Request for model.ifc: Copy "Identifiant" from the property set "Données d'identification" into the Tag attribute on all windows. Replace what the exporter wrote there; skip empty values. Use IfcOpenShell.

First a look at what the model holds.

```python
import ifcopenshell
import ifcopenshell.util.element

model = ifcopenshell.open("model.ifc")
print(model.schema)
windows = model.by_type("IfcWindow")
print(len(windows), "windows")
for e in windows[:8]:
    source = ifcopenshell.util.element.get_pset(e, "Données d'identification", "Identifiant")
    target = e.Tag
    print(e.id(), repr(source), repr(target), sep=" | ")
```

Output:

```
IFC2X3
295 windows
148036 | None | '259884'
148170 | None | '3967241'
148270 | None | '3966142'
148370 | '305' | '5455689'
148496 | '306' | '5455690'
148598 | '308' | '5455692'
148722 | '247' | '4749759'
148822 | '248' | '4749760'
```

```python
import ifcopenshell
import ifcopenshell.util.element

model = ifcopenshell.open("model.ifc")

count = 0
for e in model.by_type("IfcWindow"):
    value = ifcopenshell.util.element.get_pset(e, "Données d'identification", "Identifiant")
    current = e.Tag
    if not value or not value.strip() or current == value:
        continue
    e.Tag = value
    count += 1

print(count, "windows updated")

model.write("model_edited.ifc")
```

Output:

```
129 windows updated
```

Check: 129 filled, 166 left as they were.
